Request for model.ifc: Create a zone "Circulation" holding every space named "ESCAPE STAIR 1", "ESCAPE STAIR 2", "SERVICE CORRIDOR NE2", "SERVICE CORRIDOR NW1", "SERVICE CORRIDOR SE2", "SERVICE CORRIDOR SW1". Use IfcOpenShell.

First a look at what the model holds.

```python
import ifcopenshell

model = ifcopenshell.open("model.ifc")
print(model.schema)
seen = {}
for space in model.by_type("IfcSpace"):
    seen[space.LongName] = seen.get(space.LongName, 0) + 1
for name, count in sorted(seen.items(), key=str):
    print(count, "x", name)
print("zones:", [z.Name for z in model.by_type("IfcZone")][:20])
```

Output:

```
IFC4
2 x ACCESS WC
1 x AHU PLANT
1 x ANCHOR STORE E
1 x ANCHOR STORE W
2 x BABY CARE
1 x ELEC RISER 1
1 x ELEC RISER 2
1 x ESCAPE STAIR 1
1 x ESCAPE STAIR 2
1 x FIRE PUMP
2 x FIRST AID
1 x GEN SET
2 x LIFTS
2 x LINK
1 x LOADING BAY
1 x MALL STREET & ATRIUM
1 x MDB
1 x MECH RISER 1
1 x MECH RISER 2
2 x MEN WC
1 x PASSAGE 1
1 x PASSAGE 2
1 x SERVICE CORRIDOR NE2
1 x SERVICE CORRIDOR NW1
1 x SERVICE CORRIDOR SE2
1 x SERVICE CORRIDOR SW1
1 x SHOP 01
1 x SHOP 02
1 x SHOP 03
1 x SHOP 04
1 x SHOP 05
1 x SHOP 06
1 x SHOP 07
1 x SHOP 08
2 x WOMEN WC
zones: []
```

```python
import ifcopenshell
import ifcopenshell.api.group
import ifcopenshell.api.root

model = ifcopenshell.open("model.ifc")

names = {"ESCAPE STAIR 1", "ESCAPE STAIR 2", "SERVICE CORRIDOR NE2", "SERVICE CORRIDOR NW1", "SERVICE CORRIDOR SE2", "SERVICE CORRIDOR SW1"}
spaces = [s for s in model.by_type("IfcSpace") if s.LongName in names]

zone = ifcopenshell.api.root.create_entity(model, ifc_class="IfcZone", name="Circulation")
ifcopenshell.api.group.assign_group(model, products=spaces, group=zone)
print(len(spaces), "spaces in", zone.Name)

model.write("model_rev.ifc")
```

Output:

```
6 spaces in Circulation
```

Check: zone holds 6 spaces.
